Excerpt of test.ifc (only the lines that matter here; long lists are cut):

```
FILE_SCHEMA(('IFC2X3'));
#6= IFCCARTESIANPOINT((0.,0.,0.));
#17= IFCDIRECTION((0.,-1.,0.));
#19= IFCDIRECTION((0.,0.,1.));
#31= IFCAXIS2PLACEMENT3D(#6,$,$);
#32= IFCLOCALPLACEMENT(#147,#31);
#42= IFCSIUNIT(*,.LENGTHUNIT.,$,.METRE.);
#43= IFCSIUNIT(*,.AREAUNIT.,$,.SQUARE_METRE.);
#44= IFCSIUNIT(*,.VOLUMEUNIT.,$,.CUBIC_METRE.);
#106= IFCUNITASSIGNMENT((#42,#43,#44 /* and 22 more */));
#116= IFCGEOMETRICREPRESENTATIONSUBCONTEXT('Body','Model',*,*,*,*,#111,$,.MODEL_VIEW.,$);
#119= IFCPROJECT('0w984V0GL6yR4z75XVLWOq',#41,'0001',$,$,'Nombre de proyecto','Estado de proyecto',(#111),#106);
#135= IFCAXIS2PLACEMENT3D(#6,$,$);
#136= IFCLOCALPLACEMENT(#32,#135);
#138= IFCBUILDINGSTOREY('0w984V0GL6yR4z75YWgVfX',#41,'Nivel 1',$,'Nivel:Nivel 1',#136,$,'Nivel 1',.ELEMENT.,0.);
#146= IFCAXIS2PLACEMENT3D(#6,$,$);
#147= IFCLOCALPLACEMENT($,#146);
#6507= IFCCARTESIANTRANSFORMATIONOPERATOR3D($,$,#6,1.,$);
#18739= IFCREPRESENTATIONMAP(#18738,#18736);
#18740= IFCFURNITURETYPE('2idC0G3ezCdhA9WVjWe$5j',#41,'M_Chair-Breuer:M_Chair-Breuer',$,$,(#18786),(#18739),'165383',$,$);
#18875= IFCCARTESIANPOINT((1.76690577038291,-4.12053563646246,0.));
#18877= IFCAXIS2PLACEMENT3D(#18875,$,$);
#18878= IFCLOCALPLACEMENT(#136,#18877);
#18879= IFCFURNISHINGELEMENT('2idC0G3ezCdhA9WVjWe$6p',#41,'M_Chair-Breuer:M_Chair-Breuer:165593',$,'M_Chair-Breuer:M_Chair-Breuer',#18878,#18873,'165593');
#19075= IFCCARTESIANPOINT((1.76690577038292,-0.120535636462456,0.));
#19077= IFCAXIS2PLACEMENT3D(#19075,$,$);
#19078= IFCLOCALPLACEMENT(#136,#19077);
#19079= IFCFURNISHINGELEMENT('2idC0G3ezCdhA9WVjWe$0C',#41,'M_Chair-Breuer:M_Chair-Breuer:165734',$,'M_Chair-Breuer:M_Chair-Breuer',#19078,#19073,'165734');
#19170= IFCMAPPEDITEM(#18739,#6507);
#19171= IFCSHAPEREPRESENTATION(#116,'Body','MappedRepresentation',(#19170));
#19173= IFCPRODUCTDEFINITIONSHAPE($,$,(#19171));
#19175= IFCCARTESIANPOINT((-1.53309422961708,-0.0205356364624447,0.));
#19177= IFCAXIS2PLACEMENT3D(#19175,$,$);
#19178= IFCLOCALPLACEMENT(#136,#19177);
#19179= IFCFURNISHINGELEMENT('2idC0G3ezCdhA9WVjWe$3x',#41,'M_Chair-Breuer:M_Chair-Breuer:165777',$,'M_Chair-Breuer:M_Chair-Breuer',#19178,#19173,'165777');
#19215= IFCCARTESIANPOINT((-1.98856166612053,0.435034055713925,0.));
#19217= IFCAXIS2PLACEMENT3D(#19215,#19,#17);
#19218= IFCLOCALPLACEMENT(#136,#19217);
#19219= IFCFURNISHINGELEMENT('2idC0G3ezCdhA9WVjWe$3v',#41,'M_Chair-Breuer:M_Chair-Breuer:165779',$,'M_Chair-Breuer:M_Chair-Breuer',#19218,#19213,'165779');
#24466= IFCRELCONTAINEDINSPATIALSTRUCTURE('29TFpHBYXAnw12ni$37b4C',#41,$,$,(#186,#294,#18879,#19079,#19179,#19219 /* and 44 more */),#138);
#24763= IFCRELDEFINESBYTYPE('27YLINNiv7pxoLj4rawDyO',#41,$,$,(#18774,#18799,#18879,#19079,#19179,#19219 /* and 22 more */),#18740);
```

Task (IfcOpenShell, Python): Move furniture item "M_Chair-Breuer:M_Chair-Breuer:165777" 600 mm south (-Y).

```python
import ifcopenshell
import ifcopenshell.api.geometry
import ifcopenshell.util.placement
import ifcopenshell.util.unit

model = ifcopenshell.open("test.ifc")
unit_scale = ifcopenshell.util.unit.calculate_unit_scale(model)

item = model.by_id(19179)
matrix = ifcopenshell.util.placement.get_local_placement(item.ObjectPlacement)
matrix[1, 3] -= 0.6 / unit_scale
ifcopenshell.api.geometry.edit_object_placement(model, product=item, matrix=matrix, is_si=False)

print(ifcopenshell.util.placement.get_local_placement(item.ObjectPlacement).round(3) + 0.0)

model.write("test_v2.ifc")
```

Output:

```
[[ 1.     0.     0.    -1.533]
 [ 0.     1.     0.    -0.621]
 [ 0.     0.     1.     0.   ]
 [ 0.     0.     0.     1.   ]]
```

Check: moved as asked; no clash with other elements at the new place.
